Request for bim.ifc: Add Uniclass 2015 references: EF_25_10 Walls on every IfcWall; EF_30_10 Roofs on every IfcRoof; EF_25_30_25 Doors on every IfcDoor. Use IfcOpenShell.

First a look at what the model holds.

```python
import ifcopenshell

model = ifcopenshell.open("bim.ifc")
print(model.schema)
print("classifications:", [c.Name for c in model.by_type("IfcClassification")])
for ifc_class in ("IfcDoor", "IfcRoof", "IfcStair", "IfcWall", "IfcWindow"):
    print(ifc_class, len(model.by_type(ifc_class)))
```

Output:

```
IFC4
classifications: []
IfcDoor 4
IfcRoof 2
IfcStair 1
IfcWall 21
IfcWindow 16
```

```python
import ifcopenshell
import ifcopenshell.api.classification

model = ifcopenshell.open("bim.ifc")

system = ifcopenshell.api.classification.add_classification(model, classification="Uniclass 2015")

codes = {
    "IfcWall": ("EF_25_10", "Walls"),
    "IfcRoof": ("EF_30_10", "Roofs"),
    "IfcDoor": ("EF_25_30_25", "Doors"),
}
for ifc_class, (code, name) in codes.items():
    products = model.by_type(ifc_class)
    ifcopenshell.api.classification.add_reference(
        model, products=products, classification=system, identification=code, name=name
    )
    print(code, len(products))

model.write("bim_v2.ifc")
```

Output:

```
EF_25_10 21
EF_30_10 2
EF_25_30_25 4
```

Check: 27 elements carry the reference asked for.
